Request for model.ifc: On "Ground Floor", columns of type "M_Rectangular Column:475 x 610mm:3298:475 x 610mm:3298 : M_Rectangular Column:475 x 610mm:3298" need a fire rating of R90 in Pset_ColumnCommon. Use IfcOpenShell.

First a look at what the model holds.

```python
import ifcopenshell
import ifcopenshell.util.element

model = ifcopenshell.open("model.ifc")
print(model.schema)
storey = next(s for s in model.by_type("IfcBuildingStorey") if s.Name == "Ground Floor")
columns = [e for e in ifcopenshell.util.element.get_decomposition(storey) if e.is_a("IfcColumn")]
seen = {}
for e in columns:
    element_type = ifcopenshell.util.element.get_type(e)
    key = (element_type.Name if element_type != e and element_type else None, ifcopenshell.util.element.get_pset(e, "Pset_ColumnCommon", "FireRating"))
    seen[key] = seen.get(key, 0) + 1
for (name, value), count in sorted(seen.items(), key=str):
    print(count, "x", name, "|", value)
```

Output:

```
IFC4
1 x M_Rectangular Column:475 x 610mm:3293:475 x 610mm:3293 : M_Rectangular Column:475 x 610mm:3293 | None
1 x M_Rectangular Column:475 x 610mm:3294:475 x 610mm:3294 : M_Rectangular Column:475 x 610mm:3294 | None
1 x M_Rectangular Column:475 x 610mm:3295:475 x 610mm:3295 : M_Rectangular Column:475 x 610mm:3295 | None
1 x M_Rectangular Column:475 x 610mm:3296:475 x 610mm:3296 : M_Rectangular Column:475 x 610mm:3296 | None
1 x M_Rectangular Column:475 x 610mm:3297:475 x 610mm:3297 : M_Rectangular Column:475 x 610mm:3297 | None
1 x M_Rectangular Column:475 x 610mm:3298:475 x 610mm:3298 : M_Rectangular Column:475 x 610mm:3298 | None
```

```python
import ifcopenshell
import ifcopenshell.api.pset
import ifcopenshell.util.element

model = ifcopenshell.open("model.ifc")

storey = next(s for s in model.by_type("IfcBuildingStorey") if s.Name == "Ground Floor")
columns = [e for e in ifcopenshell.util.element.get_decomposition(storey) if e.is_a("IfcColumn")]

count = 0
for e in columns:
    element_type = ifcopenshell.util.element.get_type(e)
    if element_type in (None, e) or element_type.Name != "M_Rectangular Column:475 x 610mm:3298:475 x 610mm:3298 : M_Rectangular Column:475 x 610mm:3298":
        continue
    # add_pset returns the element's existing set when there is one.
    pset = ifcopenshell.api.pset.add_pset(model, product=e, name="Pset_ColumnCommon")
    ifcopenshell.api.pset.edit_pset(model, pset=pset, properties={"FireRating": "R90"})
    count += 1

print(count, "columns updated")

model.write("model_rev.ifc")
```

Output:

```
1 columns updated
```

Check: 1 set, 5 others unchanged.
